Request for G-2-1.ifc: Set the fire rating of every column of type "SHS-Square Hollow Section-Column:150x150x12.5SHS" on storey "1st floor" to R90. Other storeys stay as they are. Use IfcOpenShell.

First a look at what the model holds.

```python
import ifcopenshell
import ifcopenshell.util.element

model = ifcopenshell.open("G-2-1.ifc")
print(model.schema)
storey = next(s for s in model.by_type("IfcBuildingStorey") if s.Name == "1st floor")
columns = [e for e in ifcopenshell.util.element.get_decomposition(storey) if e.is_a("IfcColumn")]
seen = {}
for e in columns:
    element_type = ifcopenshell.util.element.get_type(e)
    key = (element_type.Name if element_type != e and element_type else None, ifcopenshell.util.element.get_pset(e, "Pset_ColumnCommon", "FireRating"))
    seen[key] = seen.get(key, 0) + 1
for (name, value), count in sorted(seen.items(), key=str):
    print(count, "x", name, "|", value)
```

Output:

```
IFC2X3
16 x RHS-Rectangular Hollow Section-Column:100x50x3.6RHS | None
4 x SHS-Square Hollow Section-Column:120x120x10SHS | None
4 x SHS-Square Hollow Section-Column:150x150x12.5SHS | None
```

```python
import ifcopenshell
import ifcopenshell.api.pset
import ifcopenshell.util.element

model = ifcopenshell.open("G-2-1.ifc")

storey = next(s for s in model.by_type("IfcBuildingStorey") if s.Name == "1st floor")
columns = [e for e in ifcopenshell.util.element.get_decomposition(storey) if e.is_a("IfcColumn")]

count = 0
for e in columns:
    element_type = ifcopenshell.util.element.get_type(e)
    if element_type in (None, e) or element_type.Name != "SHS-Square Hollow Section-Column:150x150x12.5SHS":
        continue
    # add_pset returns the element's existing set when there is one.
    pset = ifcopenshell.api.pset.add_pset(model, product=e, name="Pset_ColumnCommon")
    ifcopenshell.api.pset.edit_pset(model, pset=pset, properties={"FireRating": "R90"})
    count += 1

print(count, "columns updated")

model.write("G-2-1_v2.ifc")
```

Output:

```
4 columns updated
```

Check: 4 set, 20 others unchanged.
